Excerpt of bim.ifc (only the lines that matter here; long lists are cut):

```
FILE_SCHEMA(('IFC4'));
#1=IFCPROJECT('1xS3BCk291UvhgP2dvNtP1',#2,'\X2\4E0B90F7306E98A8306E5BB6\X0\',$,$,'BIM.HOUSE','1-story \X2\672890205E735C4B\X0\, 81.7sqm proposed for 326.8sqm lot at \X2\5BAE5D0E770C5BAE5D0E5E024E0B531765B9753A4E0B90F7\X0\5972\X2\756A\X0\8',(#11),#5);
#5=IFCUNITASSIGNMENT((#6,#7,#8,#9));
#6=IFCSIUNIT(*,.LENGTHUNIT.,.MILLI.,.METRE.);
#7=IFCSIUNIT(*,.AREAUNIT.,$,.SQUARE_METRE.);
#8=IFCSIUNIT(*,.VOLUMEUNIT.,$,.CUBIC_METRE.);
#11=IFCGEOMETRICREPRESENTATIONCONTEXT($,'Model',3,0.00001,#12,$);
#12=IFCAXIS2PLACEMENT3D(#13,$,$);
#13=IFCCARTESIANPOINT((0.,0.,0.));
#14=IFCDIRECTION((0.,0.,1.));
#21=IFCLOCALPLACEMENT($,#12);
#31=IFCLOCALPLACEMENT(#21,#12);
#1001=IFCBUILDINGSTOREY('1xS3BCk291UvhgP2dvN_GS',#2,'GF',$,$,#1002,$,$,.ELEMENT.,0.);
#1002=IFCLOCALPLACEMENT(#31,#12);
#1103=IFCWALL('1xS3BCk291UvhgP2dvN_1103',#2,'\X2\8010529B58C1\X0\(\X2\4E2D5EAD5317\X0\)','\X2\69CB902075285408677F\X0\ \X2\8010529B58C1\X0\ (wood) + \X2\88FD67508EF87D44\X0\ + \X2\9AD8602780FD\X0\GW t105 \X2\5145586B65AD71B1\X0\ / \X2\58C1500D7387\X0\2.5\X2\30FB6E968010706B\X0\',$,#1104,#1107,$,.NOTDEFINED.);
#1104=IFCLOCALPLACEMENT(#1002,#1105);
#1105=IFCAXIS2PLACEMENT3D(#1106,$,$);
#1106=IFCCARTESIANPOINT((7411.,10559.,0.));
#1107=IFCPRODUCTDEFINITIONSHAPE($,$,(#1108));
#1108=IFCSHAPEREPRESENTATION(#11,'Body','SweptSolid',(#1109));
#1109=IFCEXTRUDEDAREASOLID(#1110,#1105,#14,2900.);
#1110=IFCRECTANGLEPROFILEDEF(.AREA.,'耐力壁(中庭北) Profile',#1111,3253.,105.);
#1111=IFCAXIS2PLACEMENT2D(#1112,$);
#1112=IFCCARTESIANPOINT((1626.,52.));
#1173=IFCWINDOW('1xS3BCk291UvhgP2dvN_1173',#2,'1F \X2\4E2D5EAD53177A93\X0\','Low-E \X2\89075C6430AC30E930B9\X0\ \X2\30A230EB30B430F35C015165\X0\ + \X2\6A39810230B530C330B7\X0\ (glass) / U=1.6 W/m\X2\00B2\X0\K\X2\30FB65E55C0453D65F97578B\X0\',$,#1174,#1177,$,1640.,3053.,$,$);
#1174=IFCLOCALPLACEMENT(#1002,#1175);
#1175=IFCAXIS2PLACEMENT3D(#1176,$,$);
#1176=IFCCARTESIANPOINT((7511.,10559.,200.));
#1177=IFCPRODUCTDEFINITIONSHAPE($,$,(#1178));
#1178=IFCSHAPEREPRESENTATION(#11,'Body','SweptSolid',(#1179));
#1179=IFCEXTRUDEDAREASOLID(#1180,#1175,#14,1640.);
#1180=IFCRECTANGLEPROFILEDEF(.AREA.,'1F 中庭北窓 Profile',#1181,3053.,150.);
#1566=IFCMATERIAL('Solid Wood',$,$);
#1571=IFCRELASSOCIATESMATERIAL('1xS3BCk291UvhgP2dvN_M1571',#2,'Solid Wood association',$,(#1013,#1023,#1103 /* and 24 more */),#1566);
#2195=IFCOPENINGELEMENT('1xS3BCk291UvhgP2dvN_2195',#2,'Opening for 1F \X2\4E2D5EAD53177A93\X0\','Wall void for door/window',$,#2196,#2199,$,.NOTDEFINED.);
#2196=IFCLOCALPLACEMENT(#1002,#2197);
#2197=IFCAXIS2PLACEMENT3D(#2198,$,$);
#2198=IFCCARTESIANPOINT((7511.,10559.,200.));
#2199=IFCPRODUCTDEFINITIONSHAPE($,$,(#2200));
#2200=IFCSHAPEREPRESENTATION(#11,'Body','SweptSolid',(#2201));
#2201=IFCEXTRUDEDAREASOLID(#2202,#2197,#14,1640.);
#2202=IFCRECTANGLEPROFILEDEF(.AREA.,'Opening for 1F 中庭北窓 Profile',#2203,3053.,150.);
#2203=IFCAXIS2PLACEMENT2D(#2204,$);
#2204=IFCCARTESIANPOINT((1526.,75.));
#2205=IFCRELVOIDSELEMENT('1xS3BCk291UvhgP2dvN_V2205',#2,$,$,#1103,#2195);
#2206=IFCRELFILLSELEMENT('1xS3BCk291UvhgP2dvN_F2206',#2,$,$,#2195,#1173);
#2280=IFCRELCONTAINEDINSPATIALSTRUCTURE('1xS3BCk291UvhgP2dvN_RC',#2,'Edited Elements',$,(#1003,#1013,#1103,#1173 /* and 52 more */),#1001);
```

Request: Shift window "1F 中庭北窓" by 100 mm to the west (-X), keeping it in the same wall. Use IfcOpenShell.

```python
import ifcopenshell
import ifcopenshell.api.geometry
import ifcopenshell.util.placement
import ifcopenshell.util.unit

model = ifcopenshell.open("bim.ifc")
unit_scale = ifcopenshell.util.unit.calculate_unit_scale(model)

window = model.by_guid("1xS3BCk291UvhgP2dvN_1173")
opening = window.FillsVoids[0].RelatingOpeningElement
wall = opening.VoidsElements[0].RelatingBuildingElement

wall_matrix = ifcopenshell.util.placement.get_local_placement(wall.ObjectPlacement)
shift = wall_matrix[:3, 0] * -0.1 / unit_scale
before = ifcopenshell.util.placement.get_local_placement(window.ObjectPlacement)[:3, 3].copy()

# The window is not placed relative to its opening, so move both.
for product in (opening, window):
    matrix = ifcopenshell.util.placement.get_local_placement(product.ObjectPlacement)
    matrix[:3, 3] += shift
    ifcopenshell.api.geometry.edit_object_placement(model, product=product, matrix=matrix, is_si=False)

after = ifcopenshell.util.placement.get_local_placement(window.ObjectPlacement)[:3, 3]
print("window moved by", (after - before).round(3) + 0.0)

model.write("bim_updated.ifc")
```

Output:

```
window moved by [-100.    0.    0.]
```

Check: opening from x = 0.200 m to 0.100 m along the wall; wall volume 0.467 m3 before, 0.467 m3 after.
